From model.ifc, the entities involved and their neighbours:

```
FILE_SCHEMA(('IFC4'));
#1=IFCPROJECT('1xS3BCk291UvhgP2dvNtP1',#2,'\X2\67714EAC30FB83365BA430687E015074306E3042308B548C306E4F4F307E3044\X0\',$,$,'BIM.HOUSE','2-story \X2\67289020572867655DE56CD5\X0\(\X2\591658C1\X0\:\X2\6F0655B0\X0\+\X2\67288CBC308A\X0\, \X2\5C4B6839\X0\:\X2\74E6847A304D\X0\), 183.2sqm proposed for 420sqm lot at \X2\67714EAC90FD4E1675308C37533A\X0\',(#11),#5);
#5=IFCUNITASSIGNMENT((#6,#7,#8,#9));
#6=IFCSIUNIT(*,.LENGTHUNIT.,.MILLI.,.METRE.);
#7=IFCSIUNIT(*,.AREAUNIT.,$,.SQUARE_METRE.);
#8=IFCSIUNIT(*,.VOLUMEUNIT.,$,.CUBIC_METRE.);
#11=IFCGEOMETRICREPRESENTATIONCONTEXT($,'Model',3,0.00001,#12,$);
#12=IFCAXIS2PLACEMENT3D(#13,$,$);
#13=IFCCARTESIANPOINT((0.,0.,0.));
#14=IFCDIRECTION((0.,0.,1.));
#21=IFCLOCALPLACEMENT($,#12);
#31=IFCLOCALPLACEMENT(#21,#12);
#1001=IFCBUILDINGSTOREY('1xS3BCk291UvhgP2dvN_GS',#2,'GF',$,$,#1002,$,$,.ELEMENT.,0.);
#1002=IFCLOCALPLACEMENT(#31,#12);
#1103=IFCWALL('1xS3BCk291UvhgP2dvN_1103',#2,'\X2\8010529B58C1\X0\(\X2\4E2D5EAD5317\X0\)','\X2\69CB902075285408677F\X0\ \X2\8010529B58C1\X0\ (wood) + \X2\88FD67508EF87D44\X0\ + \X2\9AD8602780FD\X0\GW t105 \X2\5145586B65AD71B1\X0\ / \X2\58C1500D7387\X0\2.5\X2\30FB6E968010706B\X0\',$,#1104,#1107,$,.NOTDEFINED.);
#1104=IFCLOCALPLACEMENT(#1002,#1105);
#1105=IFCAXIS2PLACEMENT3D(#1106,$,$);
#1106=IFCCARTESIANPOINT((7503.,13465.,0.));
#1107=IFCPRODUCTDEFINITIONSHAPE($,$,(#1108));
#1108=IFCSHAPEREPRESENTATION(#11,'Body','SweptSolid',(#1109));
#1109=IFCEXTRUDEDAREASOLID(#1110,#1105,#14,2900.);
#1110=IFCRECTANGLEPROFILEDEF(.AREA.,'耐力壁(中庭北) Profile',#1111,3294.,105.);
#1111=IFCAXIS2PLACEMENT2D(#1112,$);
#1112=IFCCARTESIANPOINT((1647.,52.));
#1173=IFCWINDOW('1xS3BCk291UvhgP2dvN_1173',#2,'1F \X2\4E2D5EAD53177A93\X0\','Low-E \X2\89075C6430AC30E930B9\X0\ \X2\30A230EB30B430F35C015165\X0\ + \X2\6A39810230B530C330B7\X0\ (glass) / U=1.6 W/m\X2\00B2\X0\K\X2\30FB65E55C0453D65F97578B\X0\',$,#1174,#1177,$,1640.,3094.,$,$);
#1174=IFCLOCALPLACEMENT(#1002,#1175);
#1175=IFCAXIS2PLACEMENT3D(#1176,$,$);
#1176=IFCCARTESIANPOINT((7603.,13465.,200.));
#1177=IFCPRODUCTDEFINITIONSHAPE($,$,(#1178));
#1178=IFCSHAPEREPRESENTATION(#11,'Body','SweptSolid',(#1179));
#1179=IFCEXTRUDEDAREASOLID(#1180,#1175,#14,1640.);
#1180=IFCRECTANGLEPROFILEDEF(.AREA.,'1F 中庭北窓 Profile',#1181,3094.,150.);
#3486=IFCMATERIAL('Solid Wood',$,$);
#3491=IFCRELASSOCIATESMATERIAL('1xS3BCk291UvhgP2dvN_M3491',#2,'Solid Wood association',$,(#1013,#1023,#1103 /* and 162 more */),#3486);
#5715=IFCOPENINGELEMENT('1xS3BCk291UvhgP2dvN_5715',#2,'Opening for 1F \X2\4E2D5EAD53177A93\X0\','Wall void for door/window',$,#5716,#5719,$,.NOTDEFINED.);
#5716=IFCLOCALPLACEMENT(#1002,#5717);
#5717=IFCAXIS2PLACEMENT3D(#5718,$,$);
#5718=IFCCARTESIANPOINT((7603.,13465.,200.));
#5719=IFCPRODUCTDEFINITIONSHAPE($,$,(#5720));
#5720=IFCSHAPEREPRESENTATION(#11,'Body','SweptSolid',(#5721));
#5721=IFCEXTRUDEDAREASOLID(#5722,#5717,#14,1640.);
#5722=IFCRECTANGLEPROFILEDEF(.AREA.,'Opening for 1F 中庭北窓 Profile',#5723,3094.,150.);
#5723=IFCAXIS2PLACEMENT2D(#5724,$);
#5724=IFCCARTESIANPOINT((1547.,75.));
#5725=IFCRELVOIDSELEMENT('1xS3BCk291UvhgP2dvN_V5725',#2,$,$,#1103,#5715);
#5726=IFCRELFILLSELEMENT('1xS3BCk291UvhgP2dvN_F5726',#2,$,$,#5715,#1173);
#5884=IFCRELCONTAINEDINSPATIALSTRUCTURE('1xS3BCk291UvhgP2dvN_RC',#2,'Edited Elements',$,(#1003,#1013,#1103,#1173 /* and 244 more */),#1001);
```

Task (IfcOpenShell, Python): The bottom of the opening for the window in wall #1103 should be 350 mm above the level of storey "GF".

```python
import numpy as np
import ifcopenshell
import ifcopenshell.api.geometry
import ifcopenshell.geom
import ifcopenshell.util.element
import ifcopenshell.util.placement
import ifcopenshell.util.shape
import ifcopenshell.util.unit

model = ifcopenshell.open("model.ifc")
unit_scale = ifcopenshell.util.unit.calculate_unit_scale(model)

window = model.by_guid("1xS3BCk291UvhgP2dvN_1173")
opening = window.FillsVoids[0].RelatingOpeningElement
storey = ifcopenshell.util.element.get_container(window, ifc_class="IfcBuildingStorey")
level = ifcopenshell.util.placement.get_local_placement(storey.ObjectPlacement)[2, 3]

# The opening's origin need not be at the sill, so measure its lowest point.
shape = ifcopenshell.geom.create_shape(ifcopenshell.geom.settings(), opening)
bottom = ifcopenshell.util.shape.get_shape_bottom_elevation(shape, shape.geometry) / unit_scale
dz = level + 0.35 / unit_scale - bottom

shift = np.array([0.0, 0.0, dz])
# The window is not placed relative to its opening, so move both.
for product in (opening, window):
    matrix = ifcopenshell.util.placement.get_local_placement(product.ObjectPlacement)
    matrix[:3, 3] += shift
    ifcopenshell.api.geometry.edit_object_placement(model, product=product, matrix=matrix, is_si=False)

print(f"moved by {dz * unit_scale:+.3f} m")

model.write("model_edited.ifc")
```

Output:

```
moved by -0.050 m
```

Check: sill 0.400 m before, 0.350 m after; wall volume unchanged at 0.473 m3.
